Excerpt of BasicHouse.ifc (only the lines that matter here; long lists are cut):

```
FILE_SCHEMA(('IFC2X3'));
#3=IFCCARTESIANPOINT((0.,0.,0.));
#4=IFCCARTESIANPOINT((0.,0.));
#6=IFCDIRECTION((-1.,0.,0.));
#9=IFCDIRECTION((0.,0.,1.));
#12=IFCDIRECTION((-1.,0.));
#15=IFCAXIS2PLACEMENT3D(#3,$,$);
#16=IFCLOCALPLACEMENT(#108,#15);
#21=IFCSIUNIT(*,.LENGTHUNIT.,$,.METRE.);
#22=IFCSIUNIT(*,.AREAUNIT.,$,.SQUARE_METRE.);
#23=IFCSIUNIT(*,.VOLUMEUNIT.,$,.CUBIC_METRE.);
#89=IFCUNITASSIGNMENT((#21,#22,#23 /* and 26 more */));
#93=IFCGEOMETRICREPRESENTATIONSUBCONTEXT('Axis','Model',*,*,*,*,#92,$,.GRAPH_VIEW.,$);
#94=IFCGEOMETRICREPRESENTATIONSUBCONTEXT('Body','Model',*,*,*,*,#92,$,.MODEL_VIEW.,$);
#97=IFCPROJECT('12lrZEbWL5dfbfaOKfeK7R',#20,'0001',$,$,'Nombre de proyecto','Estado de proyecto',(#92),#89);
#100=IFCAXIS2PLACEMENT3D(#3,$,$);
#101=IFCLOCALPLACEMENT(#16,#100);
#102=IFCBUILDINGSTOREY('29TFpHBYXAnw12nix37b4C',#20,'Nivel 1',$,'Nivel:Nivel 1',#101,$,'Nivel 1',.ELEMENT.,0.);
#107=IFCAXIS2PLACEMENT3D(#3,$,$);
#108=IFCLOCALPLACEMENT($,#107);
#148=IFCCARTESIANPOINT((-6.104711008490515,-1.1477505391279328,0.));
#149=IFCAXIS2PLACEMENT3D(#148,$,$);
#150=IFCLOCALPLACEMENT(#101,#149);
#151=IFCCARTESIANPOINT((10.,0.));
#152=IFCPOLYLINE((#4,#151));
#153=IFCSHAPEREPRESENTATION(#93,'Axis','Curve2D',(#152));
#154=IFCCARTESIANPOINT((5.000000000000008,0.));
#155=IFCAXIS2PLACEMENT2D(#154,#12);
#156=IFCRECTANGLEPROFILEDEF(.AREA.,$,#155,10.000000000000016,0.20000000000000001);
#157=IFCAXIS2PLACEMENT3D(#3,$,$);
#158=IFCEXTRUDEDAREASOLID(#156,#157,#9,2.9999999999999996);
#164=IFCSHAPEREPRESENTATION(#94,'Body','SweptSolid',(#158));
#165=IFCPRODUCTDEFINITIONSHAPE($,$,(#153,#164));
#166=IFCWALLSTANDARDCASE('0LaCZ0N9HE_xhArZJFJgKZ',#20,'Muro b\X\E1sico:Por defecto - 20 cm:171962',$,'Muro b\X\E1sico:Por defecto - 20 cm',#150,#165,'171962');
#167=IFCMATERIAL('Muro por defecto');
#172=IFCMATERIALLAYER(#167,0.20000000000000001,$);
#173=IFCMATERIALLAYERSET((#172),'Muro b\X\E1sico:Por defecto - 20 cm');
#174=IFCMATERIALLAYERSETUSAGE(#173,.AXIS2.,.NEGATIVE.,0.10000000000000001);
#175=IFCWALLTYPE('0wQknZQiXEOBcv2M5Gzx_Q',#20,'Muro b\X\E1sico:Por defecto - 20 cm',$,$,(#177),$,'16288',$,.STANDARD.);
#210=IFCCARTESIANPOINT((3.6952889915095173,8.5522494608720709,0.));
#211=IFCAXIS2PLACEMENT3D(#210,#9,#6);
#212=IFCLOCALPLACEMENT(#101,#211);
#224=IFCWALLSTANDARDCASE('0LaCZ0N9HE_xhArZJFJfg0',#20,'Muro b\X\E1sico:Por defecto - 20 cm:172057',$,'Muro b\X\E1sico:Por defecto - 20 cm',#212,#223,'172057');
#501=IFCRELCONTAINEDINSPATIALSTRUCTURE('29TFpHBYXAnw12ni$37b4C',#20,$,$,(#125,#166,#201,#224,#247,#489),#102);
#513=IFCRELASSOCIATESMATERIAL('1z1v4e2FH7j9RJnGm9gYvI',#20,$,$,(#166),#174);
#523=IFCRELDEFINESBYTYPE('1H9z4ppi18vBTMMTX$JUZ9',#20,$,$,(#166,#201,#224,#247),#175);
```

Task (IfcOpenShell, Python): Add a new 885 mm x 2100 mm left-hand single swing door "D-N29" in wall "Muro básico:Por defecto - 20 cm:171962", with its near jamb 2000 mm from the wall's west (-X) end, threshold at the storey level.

```python
import numpy as np
import ifcopenshell
import ifcopenshell.api.feature
import ifcopenshell.api.geometry
import ifcopenshell.api.root
import ifcopenshell.api.spatial
import ifcopenshell.api.type
import ifcopenshell.geom
import ifcopenshell.util.element
import ifcopenshell.util.placement
import ifcopenshell.util.representation
import ifcopenshell.util.shape
import ifcopenshell.util.unit

model = ifcopenshell.open("BasicHouse.ifc")
unit_scale = ifcopenshell.util.unit.calculate_unit_scale(model)
settings = ifcopenshell.geom.settings()


def volume(element):
    """Net volume in cubic metres, openings subtracted."""
    shape = ifcopenshell.geom.create_shape(settings, element)
    return ifcopenshell.util.shape.get_volume(shape.geometry)


wall = model.by_guid("0LaCZ0N9HE_xhArZJFJgKZ")
storey = ifcopenshell.util.element.get_container(wall, ifc_class="IfcBuildingStorey")
context = ifcopenshell.util.representation.get_context(model, "Model", "Body", "MODEL_VIEW")
before = volume(wall)

width, height, from_end, sill = 0.885, 2.1, 2, 0.0  # metres

# The wall runs along its own X axis, and the end named is its -X end.
wall_shape = ifcopenshell.geom.create_shape(settings, wall)
x, y, z = ifcopenshell.util.shape.get_vertices(wall_shape.geometry).T
start = x.min() + from_end
face, thickness = float(y.min()), float(y.max() - y.min())
wall_matrix = ifcopenshell.util.placement.get_local_placement(wall.ObjectPlacement)
level = ifcopenshell.util.placement.get_local_placement(storey.ObjectPlacement)[2, 3]


def in_wall(x, y):
    """Placement at x, y metres in the wall's axes, at sill height."""
    matrix = wall_matrix.copy()
    matrix[:, 3] = wall_matrix @ np.array([x / unit_scale, y / unit_scale, 0.0, 1.0])
    matrix[2, 3] = level + sill / unit_scale
    return matrix


# Opening: a box that overshoots both wall faces by 50 mm.
opening = ifcopenshell.api.root.create_entity(model, ifc_class="IfcOpeningElement")
box = ifcopenshell.api.geometry.add_wall_representation(
    model, context=context, length=width, height=height, thickness=thickness + 0.1
)
ifcopenshell.api.geometry.assign_representation(model, product=opening, representation=box)
ifcopenshell.api.geometry.edit_object_placement(model, product=opening, matrix=in_wall(start, face - 0.05), is_si=False)
ifcopenshell.api.feature.add_feature(model, feature=opening, element=wall)

door = ifcopenshell.api.root.create_entity(model, ifc_class="IfcDoor", name="D-N29")
door.OverallWidth, door.OverallHeight = width / unit_scale, height / unit_scale
body = ifcopenshell.api.geometry.add_door_representation(
    model,
    context=context,
    overall_width=door.OverallWidth,
    overall_height=door.OverallHeight,
    operation_type="SINGLE_SWING_LEFT",
    lining_properties={"LiningDepth": thickness / unit_scale, "ThresholdDepth": thickness / unit_scale},
)
ifcopenshell.api.geometry.assign_representation(model, product=door, representation=body)
ifcopenshell.api.spatial.assign_container(model, products=[door], relating_structure=storey)
fills = ifcopenshell.api.feature.add_filling(model, opening=opening, element=door)
fills.OwnerHistory = door.OwnerHistory  # required in IFC2X3

# IFC2X3 keeps the operation on the door style.
style = ifcopenshell.api.root.create_entity(model, ifc_class="IfcDoorStyle", name="D-N29")
style.OperationType, style.ConstructionType = "SINGLE_SWING_LEFT", "NOTDEFINED"
style.ParameterTakesPrecedence = style.Sizeable = False
ifcopenshell.api.type.assign_type(model, related_objects=[door], relating_type=style)

# The lining spans the wall, so the door starts at the wall face.
ifcopenshell.api.geometry.edit_object_placement(model, product=door, matrix=in_wall(start, face), is_si=False)

after = volume(wall)

print(f"wall volume {before:.3f} -> {after:.3f} m3")

model.write("BasicHouse_updated.ifc")
```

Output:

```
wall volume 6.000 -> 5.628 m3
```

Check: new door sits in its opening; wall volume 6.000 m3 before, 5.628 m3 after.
